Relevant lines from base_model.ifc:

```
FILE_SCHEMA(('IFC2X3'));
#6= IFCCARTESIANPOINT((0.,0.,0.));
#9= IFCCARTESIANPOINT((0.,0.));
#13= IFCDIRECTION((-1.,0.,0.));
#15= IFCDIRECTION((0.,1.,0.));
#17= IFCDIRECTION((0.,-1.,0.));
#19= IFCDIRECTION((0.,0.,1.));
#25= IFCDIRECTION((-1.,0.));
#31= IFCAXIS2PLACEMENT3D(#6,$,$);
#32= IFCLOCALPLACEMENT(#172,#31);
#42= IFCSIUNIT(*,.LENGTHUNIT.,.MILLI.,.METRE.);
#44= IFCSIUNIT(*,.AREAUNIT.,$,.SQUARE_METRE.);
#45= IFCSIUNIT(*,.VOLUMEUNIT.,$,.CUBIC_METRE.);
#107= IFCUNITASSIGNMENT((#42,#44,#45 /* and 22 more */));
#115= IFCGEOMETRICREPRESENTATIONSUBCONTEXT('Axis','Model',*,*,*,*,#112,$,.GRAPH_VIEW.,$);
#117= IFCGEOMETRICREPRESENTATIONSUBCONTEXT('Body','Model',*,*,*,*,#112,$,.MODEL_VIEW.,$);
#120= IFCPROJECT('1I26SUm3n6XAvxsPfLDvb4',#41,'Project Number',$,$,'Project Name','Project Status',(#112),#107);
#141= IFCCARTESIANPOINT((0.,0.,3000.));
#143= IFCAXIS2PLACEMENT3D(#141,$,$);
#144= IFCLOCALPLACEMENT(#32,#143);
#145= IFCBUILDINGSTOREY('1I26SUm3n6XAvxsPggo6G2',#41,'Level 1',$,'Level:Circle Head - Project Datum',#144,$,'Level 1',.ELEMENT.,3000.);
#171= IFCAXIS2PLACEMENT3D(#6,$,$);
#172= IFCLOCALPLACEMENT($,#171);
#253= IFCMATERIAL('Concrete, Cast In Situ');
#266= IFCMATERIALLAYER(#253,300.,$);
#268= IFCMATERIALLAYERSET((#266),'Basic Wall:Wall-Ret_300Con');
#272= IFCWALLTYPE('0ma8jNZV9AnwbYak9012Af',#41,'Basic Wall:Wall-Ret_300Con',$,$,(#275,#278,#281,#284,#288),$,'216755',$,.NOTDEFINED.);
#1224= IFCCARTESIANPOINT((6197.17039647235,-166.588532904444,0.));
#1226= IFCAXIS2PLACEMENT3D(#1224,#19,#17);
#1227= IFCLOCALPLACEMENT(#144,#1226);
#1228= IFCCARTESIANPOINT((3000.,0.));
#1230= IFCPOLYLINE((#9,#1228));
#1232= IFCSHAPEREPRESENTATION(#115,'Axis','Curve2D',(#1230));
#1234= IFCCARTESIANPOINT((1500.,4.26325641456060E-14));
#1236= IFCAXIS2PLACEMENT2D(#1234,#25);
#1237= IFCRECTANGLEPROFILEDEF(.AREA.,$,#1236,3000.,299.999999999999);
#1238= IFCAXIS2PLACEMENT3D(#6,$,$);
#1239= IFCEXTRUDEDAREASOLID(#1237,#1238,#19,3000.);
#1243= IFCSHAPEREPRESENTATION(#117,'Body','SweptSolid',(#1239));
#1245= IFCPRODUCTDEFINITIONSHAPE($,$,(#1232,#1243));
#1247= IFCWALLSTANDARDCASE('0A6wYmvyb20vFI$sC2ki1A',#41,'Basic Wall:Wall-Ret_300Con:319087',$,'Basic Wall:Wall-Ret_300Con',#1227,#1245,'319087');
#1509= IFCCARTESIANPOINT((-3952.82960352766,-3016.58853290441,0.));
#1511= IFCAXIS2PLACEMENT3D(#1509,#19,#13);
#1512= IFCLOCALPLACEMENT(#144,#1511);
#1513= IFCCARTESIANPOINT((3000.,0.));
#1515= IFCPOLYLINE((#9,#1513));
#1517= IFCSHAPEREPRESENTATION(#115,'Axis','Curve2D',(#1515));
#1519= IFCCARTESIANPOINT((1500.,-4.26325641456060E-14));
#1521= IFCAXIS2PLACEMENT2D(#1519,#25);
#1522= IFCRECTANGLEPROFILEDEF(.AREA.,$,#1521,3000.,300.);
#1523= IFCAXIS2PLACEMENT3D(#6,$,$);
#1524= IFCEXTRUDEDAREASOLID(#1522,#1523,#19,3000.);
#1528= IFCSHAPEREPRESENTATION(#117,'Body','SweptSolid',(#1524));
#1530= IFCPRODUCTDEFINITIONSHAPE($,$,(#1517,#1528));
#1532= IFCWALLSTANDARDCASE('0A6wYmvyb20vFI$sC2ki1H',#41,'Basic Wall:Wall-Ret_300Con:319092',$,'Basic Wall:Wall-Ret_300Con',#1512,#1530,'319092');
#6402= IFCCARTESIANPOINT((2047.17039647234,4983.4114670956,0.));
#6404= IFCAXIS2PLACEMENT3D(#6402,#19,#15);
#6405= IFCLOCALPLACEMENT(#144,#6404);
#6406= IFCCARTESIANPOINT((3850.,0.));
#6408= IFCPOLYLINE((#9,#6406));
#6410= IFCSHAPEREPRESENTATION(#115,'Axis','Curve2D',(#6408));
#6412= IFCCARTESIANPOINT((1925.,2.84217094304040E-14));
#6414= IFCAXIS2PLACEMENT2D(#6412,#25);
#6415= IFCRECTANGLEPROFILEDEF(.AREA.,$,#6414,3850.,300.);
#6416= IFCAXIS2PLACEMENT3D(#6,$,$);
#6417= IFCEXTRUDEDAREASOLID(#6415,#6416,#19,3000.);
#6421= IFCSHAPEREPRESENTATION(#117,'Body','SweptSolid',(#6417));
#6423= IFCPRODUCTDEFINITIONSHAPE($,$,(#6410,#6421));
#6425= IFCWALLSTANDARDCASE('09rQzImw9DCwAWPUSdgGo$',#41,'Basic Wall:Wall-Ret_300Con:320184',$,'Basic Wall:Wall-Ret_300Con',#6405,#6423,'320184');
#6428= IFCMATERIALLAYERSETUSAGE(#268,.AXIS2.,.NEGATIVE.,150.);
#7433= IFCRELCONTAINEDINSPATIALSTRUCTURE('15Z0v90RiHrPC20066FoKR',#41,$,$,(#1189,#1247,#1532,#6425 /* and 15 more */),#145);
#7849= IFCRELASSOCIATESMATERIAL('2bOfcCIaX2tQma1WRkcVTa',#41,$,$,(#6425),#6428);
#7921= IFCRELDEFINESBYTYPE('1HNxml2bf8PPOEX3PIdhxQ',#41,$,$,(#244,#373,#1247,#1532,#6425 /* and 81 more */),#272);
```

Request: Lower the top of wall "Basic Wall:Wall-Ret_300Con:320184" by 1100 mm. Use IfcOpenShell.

```python
import ifcopenshell
import ifcopenshell.geom
import ifcopenshell.util.representation
import ifcopenshell.util.shape
import ifcopenshell.util.unit

model = ifcopenshell.open("base_model.ifc")
unit_scale = ifcopenshell.util.unit.calculate_unit_scale(model)
settings = ifcopenshell.geom.settings()


def volume(element):
    """Net volume in cubic metres, openings subtracted."""
    shape = ifcopenshell.geom.create_shape(settings, element)
    return ifcopenshell.util.shape.get_volume(shape.geometry)


wall = model.by_id(6425)
before = volume(wall)

body = ifcopenshell.util.representation.get_representation(wall, "Model", "Body")
solid = body.Items[0]
old_height = solid.Depth
solid.Depth -= 1.1 / unit_scale
after = volume(wall)

print(f"height {old_height:g} -> {solid.Depth:g}, volume {before:.3f} -> {after:.3f} m3")

model.write("base_model_rev.ifc")
```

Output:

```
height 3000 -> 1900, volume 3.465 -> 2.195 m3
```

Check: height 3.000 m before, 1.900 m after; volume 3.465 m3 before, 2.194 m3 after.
